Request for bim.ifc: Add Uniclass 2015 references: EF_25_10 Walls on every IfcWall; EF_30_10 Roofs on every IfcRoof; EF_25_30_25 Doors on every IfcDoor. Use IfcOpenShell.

First a look at what the model holds.

```python
import ifcopenshell

model = ifcopenshell.open("bim.ifc")
print(model.schema)
print("classifications:", [c.Name for c in model.by_type("IfcClassification")])
for ifc_class in ("IfcDoor", "IfcRoof", "IfcStair", "IfcWall", "IfcWindow"):
    print(ifc_class, len(model.by_type(ifc_class)))
```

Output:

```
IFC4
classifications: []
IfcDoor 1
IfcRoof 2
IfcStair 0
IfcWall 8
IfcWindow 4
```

```python
import ifcopenshell
import ifcopenshell.api.classification

model = ifcopenshell.open("bim.ifc")

system = ifcopenshell.api.classification.add_classification(model, classification="Uniclass 2015")

codes = {
    "IfcWall": ("EF_25_10", "Walls"),
    "IfcRoof": ("EF_30_10", "Roofs"),
    "IfcDoor": ("EF_25_30_25", "Doors"),
}
for ifc_class, (code, name) in codes.items():
    products = model.by_type(ifc_class)
    ifcopenshell.api.classification.add_reference(
        model, products=products, classification=system, identification=code, name=name
    )
    print(code, len(products))

model.write("bim_rev.ifc")
```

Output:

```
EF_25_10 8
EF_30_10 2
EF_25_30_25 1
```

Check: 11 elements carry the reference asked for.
